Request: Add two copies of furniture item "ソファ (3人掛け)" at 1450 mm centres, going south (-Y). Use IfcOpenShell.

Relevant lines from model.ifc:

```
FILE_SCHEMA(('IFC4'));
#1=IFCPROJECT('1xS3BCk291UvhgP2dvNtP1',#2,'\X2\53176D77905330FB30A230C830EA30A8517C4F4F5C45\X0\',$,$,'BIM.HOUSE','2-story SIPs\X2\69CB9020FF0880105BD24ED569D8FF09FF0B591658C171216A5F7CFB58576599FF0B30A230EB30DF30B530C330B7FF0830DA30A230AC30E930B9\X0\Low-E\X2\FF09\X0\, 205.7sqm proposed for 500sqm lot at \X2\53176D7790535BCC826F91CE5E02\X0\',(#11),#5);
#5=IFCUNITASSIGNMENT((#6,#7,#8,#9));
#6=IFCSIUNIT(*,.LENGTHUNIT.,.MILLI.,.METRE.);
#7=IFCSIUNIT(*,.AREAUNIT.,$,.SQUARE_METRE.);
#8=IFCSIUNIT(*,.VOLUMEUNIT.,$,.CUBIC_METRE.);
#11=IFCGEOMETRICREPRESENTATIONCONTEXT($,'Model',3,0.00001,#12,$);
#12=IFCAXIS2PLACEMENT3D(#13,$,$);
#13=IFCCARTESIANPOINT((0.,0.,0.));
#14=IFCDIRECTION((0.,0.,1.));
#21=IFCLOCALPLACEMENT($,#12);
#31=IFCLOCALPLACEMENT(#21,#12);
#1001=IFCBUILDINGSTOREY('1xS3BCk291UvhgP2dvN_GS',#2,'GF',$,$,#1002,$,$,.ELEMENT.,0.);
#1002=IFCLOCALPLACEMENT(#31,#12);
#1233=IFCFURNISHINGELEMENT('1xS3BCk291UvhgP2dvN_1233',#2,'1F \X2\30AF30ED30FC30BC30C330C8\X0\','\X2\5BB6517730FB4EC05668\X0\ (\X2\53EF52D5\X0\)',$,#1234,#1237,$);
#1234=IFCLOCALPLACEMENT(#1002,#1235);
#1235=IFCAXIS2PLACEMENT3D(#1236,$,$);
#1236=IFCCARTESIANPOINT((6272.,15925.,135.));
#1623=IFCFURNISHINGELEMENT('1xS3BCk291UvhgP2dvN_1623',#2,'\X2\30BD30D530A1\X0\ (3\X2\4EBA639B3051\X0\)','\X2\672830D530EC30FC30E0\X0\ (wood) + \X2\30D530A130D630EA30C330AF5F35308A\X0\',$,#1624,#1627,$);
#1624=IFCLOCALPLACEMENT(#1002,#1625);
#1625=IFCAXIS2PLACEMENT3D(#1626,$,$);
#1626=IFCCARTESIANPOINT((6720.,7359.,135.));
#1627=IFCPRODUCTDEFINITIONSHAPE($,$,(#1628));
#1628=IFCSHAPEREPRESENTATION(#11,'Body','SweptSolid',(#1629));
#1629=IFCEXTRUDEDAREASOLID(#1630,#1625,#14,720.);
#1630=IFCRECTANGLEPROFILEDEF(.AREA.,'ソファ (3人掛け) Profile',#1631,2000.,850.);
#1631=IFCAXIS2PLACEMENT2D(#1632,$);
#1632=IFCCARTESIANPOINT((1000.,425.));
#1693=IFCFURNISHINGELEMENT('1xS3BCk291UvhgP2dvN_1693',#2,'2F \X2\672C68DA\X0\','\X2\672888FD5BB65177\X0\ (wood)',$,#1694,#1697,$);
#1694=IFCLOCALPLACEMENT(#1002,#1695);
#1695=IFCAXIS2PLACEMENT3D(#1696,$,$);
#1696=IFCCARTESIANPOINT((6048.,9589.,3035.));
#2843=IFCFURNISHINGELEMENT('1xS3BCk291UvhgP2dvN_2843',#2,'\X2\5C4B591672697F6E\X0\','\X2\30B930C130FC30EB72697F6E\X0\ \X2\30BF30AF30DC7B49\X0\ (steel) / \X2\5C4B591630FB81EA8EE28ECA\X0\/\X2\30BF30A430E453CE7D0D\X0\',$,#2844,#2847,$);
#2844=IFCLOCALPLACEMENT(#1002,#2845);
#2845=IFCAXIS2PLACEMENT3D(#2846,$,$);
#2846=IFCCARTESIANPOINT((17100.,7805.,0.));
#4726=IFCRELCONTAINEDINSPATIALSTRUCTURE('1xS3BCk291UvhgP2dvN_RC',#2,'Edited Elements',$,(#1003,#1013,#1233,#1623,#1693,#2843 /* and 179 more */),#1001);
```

```python
import numpy as np
import ifcopenshell
import ifcopenshell.api.geometry
import ifcopenshell.api.root
import ifcopenshell.util.element
import ifcopenshell.util.placement
import ifcopenshell.util.unit

model = ifcopenshell.open("model.ifc")
unit_scale = ifcopenshell.util.unit.calculate_unit_scale(model)


def reuse_history(source, copy):
    """copy_class also copies each property set's owner history, people and application; keep the originals."""
    for rel in copy.IsDefinedBy:
        if rel.is_a("IfcRelDefinesByProperties") and (history := rel.RelatingPropertyDefinition.OwnerHistory):
            rel.RelatingPropertyDefinition.OwnerHistory = source.OwnerHistory
            ifcopenshell.util.element.remove_deep2(model, history)


source = model.by_guid("1xS3BCk291UvhgP2dvN_1623")
base = ifcopenshell.util.placement.get_local_placement(source.ObjectPlacement)
step = np.array([0.0, -1.0, 0.0]) * 1.45 / unit_scale

for i in range(1, 3):
    copy = ifcopenshell.api.root.copy_class(model, product=source)
    copy.Representation = ifcopenshell.util.element.copy_deep(
        model, source.Representation, exclude=["IfcGeometricRepresentationContext", "IfcRepresentationMap"]
    )
    reuse_history(source, copy)
    matrix = base.copy()
    matrix[:3, 3] += i * step
    print("added at", matrix[:3, 3].round(3) + 0.0)
    ifcopenshell.api.geometry.edit_object_placement(model, product=copy, matrix=matrix, is_si=False)

model.write("model-out.ifc")
```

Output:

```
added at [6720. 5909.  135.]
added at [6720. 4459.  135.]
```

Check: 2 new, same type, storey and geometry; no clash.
